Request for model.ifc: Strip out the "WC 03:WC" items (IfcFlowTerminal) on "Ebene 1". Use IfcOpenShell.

First a look at what the model holds.

```python
import ifcopenshell
import ifcopenshell.util.element

model = ifcopenshell.open("model.ifc")
print(model.schema)
storey = next(s for s in model.by_type("IfcBuildingStorey") if s.Name == "Ebene 1")
terminals = [e for e in ifcopenshell.util.element.get_decomposition(storey) if e.is_a("IfcFlowTerminal")]
seen = {}
for e in terminals:
    element_type = ifcopenshell.util.element.get_type(e)
    name = element_type.Name if element_type not in (None, e) else None
    seen[name] = seen.get(name, 0) + 1
for name, count in sorted(seen.items(), key=str):
    print(count, "x", name)
```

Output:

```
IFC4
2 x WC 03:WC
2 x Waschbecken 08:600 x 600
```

```python
import ifcopenshell
import ifcopenshell.api.root
import ifcopenshell.util.element

model = ifcopenshell.open("model.ifc")

storey = next(s for s in model.by_type("IfcBuildingStorey") if s.Name == "Ebene 1")
terminals = [e for e in ifcopenshell.util.element.get_decomposition(storey) if e.is_a("IfcFlowTerminal")]
targets = [e for e in terminals if (t := ifcopenshell.util.element.get_type(e)) not in (None, e) and t.Name == "WC 03:WC"]

for e in targets:
    ifcopenshell.api.root.remove_product(model, product=e)
print(len(targets), "removed")

model.write("model_updated.ifc")
```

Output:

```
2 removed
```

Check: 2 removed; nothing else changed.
